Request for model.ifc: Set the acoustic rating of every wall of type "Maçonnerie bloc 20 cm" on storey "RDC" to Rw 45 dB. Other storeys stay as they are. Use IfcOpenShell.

First a look at what the model holds.

```python
import ifcopenshell
import ifcopenshell.util.element

model = ifcopenshell.open("model.ifc")
print(model.schema)
storey = next(s for s in model.by_type("IfcBuildingStorey") if s.Name == "RDC")
walls = [e for e in ifcopenshell.util.element.get_decomposition(storey) if e.is_a("IfcWall")]
seen = {}
for e in walls:
    element_type = ifcopenshell.util.element.get_type(e)
    key = (element_type.Name if element_type != e and element_type else None, ifcopenshell.util.element.get_pset(e, "Pset_WallCommon", "AcousticRating"))
    seen[key] = seen.get(key, 0) + 1
for (name, value), count in sorted(seen.items(), key=str):
    print(count, "x", name, "|", value)
```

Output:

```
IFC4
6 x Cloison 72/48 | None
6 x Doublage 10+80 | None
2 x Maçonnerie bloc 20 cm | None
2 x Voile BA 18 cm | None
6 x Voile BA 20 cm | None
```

```python
import ifcopenshell
import ifcopenshell.api.pset
import ifcopenshell.util.element

model = ifcopenshell.open("model.ifc")

storey = next(s for s in model.by_type("IfcBuildingStorey") if s.Name == "RDC")
walls = [e for e in ifcopenshell.util.element.get_decomposition(storey) if e.is_a("IfcWall")]

count = 0
for e in walls:
    element_type = ifcopenshell.util.element.get_type(e)
    if element_type in (None, e) or element_type.Name != "Maçonnerie bloc 20 cm":
        continue
    # add_pset returns the element's existing set when there is one.
    pset = ifcopenshell.api.pset.add_pset(model, product=e, name="Pset_WallCommon")
    ifcopenshell.api.pset.edit_pset(model, pset=pset, properties={"AcousticRating": "Rw 45 dB"})
    count += 1

print(count, "walls updated")

model.write("model_v2.ifc")
```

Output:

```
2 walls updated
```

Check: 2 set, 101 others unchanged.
